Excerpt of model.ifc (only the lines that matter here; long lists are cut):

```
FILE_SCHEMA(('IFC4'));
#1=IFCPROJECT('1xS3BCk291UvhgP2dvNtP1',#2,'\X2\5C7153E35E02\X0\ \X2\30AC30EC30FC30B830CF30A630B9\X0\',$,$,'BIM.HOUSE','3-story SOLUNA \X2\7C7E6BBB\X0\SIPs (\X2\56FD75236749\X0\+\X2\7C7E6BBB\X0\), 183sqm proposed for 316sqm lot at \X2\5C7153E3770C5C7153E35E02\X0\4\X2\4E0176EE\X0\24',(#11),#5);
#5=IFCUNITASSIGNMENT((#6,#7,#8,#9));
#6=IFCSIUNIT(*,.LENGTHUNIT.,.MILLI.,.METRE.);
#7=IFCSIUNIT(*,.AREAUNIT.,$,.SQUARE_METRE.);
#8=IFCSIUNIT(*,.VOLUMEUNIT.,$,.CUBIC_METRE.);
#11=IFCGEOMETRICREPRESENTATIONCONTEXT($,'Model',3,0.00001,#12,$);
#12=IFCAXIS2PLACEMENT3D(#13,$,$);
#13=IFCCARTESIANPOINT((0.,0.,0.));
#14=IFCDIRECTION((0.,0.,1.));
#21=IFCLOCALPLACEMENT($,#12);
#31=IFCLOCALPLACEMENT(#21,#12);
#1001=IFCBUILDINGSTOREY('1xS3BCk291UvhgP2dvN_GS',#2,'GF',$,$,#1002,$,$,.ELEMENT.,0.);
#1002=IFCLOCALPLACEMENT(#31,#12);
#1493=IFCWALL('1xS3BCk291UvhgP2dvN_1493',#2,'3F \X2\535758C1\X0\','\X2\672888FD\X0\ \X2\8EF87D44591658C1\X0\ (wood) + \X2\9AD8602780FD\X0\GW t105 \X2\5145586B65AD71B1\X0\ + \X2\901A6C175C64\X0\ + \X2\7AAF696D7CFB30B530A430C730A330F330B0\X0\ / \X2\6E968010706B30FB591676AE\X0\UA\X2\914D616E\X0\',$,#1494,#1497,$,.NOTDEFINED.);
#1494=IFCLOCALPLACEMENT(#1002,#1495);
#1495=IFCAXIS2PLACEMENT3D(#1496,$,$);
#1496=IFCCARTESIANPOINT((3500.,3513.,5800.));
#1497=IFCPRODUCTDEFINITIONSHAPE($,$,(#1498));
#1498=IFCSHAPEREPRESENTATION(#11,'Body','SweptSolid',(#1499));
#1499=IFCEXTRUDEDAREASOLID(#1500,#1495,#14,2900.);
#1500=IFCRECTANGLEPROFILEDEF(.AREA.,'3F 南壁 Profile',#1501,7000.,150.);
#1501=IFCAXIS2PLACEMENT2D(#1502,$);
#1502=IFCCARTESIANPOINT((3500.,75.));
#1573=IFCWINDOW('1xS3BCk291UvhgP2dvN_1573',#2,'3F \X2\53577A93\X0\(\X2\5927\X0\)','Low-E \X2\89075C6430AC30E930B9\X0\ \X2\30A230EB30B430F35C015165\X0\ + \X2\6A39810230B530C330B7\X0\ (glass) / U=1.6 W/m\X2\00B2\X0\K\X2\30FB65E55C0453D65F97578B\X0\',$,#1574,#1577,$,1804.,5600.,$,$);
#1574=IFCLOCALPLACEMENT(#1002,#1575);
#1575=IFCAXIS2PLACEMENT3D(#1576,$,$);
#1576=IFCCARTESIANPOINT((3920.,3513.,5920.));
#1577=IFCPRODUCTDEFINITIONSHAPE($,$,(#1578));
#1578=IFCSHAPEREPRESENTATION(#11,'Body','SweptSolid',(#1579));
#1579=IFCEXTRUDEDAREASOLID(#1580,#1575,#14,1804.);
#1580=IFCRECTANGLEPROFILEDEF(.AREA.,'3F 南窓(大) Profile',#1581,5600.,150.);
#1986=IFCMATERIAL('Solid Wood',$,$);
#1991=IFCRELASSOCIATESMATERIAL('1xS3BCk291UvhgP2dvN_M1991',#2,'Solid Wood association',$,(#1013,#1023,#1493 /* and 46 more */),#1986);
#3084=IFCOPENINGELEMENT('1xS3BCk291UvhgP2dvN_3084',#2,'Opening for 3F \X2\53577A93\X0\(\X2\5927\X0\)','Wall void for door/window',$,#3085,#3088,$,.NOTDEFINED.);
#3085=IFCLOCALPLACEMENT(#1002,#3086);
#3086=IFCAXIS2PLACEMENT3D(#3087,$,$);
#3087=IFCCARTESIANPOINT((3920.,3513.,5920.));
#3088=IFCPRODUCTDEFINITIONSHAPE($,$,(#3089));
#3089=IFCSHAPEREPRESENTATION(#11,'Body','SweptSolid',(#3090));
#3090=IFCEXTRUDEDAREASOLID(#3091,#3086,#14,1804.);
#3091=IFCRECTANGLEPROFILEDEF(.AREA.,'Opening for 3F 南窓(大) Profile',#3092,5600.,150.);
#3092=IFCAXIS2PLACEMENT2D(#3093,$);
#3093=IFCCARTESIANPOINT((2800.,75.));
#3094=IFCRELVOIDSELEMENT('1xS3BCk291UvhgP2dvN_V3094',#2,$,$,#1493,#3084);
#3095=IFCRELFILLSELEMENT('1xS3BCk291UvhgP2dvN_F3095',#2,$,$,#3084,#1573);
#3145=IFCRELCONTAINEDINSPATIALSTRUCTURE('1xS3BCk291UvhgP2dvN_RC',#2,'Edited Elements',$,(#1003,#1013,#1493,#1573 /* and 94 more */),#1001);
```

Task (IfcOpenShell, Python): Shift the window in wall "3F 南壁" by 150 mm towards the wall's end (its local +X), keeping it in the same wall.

```python
import ifcopenshell
import ifcopenshell.api.geometry
import ifcopenshell.util.placement

model = ifcopenshell.open("model.ifc")

window = model.by_guid("1xS3BCk291UvhgP2dvN_1573")
opening = window.FillsVoids[0].RelatingOpeningElement
wall = opening.VoidsElements[0].RelatingBuildingElement

wall_matrix = ifcopenshell.util.placement.get_local_placement(wall.ObjectPlacement)
shift = wall_matrix[:3, 0] * 150.0
before = ifcopenshell.util.placement.get_local_placement(window.ObjectPlacement)[:3, 3].copy()

# The window is not placed relative to its opening, so move both.
for product in (opening, window):
    matrix = ifcopenshell.util.placement.get_local_placement(product.ObjectPlacement)
    matrix[:3, 3] += shift
    ifcopenshell.api.geometry.edit_object_placement(model, product=product, matrix=matrix, is_si=False)

after = ifcopenshell.util.placement.get_local_placement(window.ObjectPlacement)[:3, 3]
print("window moved by", (after - before).round(3) + 0.0)

model.write("model_edited.ifc")
```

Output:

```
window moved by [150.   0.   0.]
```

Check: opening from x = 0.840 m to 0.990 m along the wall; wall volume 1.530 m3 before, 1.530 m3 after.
